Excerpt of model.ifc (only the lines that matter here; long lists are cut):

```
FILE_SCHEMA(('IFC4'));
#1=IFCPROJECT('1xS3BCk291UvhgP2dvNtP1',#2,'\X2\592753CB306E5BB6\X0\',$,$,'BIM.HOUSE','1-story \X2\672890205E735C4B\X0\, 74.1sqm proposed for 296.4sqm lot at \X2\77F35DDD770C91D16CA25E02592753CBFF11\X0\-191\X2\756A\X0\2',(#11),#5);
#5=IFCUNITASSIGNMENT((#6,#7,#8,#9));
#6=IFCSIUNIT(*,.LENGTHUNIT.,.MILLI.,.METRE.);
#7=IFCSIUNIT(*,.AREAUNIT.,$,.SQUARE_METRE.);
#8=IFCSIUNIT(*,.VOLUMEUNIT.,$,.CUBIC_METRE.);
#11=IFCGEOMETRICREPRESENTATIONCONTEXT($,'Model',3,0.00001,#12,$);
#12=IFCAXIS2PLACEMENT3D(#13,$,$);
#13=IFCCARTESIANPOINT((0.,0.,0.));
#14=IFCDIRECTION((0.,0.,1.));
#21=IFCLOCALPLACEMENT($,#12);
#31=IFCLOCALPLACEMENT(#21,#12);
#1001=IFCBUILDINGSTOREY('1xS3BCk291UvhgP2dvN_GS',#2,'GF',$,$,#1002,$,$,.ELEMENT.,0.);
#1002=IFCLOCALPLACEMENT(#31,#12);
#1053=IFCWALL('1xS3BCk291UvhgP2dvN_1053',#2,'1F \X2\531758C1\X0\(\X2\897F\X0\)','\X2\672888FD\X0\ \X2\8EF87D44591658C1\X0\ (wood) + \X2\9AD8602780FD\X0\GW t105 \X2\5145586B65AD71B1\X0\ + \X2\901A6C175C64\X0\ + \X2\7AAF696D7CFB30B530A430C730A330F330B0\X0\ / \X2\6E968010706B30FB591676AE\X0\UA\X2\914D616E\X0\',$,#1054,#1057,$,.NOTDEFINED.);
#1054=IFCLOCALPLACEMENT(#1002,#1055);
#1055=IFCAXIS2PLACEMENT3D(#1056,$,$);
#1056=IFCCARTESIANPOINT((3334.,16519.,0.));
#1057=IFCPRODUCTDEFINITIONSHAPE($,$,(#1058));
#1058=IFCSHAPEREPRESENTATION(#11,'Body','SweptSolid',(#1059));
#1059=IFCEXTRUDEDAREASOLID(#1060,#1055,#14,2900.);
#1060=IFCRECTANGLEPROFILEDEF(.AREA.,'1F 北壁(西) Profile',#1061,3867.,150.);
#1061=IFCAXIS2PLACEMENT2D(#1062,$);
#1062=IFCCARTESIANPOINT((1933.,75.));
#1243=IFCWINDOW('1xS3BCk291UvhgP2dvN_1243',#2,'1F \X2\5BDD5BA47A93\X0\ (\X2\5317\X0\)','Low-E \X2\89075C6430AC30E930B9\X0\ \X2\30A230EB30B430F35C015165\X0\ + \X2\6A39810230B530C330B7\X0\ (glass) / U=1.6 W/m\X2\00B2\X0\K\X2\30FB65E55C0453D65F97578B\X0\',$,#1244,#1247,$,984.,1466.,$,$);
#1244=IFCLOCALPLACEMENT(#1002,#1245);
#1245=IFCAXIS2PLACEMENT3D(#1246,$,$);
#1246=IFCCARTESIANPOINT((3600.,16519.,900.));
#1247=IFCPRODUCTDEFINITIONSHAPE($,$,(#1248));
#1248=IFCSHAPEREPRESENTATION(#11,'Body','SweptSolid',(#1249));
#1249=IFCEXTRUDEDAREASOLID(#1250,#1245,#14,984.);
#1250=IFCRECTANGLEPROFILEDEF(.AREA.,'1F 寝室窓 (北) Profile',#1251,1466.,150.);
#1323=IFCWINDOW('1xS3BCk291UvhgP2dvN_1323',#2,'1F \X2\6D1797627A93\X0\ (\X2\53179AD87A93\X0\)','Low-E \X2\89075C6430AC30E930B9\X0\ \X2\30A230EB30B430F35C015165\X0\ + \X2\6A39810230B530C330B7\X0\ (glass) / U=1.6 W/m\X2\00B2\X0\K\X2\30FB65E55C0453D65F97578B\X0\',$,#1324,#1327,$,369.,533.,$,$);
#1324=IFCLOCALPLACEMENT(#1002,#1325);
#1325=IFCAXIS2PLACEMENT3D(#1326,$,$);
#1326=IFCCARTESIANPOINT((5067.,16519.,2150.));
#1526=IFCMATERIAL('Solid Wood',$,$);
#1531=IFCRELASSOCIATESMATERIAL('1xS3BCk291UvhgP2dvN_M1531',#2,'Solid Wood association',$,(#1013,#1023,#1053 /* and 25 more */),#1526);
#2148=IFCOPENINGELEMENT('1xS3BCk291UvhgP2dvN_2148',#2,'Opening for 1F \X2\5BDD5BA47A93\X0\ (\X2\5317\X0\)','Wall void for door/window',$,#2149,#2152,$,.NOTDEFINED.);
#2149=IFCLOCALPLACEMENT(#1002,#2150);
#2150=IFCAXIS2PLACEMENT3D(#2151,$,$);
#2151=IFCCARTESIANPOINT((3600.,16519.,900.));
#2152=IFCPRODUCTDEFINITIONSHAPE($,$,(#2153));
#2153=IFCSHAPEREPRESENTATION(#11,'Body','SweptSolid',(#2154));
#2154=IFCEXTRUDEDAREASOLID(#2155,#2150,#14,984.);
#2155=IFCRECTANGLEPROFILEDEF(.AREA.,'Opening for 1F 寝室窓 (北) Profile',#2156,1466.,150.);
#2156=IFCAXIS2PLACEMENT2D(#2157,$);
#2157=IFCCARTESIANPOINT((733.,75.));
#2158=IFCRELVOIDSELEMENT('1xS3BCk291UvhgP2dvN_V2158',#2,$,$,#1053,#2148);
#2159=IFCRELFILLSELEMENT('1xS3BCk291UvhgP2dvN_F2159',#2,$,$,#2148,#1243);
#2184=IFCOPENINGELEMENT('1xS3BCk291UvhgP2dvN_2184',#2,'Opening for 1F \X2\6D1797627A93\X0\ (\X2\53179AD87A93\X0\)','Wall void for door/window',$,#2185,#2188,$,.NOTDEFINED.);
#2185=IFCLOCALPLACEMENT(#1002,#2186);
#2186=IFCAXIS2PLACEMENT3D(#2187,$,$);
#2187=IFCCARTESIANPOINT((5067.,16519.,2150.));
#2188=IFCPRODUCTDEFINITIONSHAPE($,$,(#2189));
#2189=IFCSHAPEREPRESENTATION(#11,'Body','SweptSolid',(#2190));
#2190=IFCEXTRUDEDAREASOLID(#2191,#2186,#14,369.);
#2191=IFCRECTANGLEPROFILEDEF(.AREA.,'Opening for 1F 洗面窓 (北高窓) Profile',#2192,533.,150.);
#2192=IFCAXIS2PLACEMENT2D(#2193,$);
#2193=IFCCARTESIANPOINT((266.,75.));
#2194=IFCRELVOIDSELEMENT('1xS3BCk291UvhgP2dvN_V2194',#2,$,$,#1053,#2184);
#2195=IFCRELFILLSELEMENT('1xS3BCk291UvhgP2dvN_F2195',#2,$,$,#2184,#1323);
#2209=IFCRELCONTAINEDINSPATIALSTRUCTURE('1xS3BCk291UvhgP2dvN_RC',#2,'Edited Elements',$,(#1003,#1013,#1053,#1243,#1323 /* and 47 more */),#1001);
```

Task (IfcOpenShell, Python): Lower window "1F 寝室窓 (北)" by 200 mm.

```python
import numpy as np
import ifcopenshell
import ifcopenshell.api.geometry
import ifcopenshell.util.placement
import ifcopenshell.util.unit

model = ifcopenshell.open("model.ifc")
unit_scale = ifcopenshell.util.unit.calculate_unit_scale(model)

window = model.by_guid("1xS3BCk291UvhgP2dvN_1243")
opening = window.FillsVoids[0].RelatingOpeningElement
dz = -0.2 / unit_scale

shift = np.array([0.0, 0.0, dz])
# The window is not placed relative to its opening, so move both.
for product in (opening, window):
    matrix = ifcopenshell.util.placement.get_local_placement(product.ObjectPlacement)
    matrix[:3, 3] += shift
    ifcopenshell.api.geometry.edit_object_placement(model, product=product, matrix=matrix, is_si=False)

print(f"moved by {dz * unit_scale:+.3f} m")

model.write("model_updated.ifc")
```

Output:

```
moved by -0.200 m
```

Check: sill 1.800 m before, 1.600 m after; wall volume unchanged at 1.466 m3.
